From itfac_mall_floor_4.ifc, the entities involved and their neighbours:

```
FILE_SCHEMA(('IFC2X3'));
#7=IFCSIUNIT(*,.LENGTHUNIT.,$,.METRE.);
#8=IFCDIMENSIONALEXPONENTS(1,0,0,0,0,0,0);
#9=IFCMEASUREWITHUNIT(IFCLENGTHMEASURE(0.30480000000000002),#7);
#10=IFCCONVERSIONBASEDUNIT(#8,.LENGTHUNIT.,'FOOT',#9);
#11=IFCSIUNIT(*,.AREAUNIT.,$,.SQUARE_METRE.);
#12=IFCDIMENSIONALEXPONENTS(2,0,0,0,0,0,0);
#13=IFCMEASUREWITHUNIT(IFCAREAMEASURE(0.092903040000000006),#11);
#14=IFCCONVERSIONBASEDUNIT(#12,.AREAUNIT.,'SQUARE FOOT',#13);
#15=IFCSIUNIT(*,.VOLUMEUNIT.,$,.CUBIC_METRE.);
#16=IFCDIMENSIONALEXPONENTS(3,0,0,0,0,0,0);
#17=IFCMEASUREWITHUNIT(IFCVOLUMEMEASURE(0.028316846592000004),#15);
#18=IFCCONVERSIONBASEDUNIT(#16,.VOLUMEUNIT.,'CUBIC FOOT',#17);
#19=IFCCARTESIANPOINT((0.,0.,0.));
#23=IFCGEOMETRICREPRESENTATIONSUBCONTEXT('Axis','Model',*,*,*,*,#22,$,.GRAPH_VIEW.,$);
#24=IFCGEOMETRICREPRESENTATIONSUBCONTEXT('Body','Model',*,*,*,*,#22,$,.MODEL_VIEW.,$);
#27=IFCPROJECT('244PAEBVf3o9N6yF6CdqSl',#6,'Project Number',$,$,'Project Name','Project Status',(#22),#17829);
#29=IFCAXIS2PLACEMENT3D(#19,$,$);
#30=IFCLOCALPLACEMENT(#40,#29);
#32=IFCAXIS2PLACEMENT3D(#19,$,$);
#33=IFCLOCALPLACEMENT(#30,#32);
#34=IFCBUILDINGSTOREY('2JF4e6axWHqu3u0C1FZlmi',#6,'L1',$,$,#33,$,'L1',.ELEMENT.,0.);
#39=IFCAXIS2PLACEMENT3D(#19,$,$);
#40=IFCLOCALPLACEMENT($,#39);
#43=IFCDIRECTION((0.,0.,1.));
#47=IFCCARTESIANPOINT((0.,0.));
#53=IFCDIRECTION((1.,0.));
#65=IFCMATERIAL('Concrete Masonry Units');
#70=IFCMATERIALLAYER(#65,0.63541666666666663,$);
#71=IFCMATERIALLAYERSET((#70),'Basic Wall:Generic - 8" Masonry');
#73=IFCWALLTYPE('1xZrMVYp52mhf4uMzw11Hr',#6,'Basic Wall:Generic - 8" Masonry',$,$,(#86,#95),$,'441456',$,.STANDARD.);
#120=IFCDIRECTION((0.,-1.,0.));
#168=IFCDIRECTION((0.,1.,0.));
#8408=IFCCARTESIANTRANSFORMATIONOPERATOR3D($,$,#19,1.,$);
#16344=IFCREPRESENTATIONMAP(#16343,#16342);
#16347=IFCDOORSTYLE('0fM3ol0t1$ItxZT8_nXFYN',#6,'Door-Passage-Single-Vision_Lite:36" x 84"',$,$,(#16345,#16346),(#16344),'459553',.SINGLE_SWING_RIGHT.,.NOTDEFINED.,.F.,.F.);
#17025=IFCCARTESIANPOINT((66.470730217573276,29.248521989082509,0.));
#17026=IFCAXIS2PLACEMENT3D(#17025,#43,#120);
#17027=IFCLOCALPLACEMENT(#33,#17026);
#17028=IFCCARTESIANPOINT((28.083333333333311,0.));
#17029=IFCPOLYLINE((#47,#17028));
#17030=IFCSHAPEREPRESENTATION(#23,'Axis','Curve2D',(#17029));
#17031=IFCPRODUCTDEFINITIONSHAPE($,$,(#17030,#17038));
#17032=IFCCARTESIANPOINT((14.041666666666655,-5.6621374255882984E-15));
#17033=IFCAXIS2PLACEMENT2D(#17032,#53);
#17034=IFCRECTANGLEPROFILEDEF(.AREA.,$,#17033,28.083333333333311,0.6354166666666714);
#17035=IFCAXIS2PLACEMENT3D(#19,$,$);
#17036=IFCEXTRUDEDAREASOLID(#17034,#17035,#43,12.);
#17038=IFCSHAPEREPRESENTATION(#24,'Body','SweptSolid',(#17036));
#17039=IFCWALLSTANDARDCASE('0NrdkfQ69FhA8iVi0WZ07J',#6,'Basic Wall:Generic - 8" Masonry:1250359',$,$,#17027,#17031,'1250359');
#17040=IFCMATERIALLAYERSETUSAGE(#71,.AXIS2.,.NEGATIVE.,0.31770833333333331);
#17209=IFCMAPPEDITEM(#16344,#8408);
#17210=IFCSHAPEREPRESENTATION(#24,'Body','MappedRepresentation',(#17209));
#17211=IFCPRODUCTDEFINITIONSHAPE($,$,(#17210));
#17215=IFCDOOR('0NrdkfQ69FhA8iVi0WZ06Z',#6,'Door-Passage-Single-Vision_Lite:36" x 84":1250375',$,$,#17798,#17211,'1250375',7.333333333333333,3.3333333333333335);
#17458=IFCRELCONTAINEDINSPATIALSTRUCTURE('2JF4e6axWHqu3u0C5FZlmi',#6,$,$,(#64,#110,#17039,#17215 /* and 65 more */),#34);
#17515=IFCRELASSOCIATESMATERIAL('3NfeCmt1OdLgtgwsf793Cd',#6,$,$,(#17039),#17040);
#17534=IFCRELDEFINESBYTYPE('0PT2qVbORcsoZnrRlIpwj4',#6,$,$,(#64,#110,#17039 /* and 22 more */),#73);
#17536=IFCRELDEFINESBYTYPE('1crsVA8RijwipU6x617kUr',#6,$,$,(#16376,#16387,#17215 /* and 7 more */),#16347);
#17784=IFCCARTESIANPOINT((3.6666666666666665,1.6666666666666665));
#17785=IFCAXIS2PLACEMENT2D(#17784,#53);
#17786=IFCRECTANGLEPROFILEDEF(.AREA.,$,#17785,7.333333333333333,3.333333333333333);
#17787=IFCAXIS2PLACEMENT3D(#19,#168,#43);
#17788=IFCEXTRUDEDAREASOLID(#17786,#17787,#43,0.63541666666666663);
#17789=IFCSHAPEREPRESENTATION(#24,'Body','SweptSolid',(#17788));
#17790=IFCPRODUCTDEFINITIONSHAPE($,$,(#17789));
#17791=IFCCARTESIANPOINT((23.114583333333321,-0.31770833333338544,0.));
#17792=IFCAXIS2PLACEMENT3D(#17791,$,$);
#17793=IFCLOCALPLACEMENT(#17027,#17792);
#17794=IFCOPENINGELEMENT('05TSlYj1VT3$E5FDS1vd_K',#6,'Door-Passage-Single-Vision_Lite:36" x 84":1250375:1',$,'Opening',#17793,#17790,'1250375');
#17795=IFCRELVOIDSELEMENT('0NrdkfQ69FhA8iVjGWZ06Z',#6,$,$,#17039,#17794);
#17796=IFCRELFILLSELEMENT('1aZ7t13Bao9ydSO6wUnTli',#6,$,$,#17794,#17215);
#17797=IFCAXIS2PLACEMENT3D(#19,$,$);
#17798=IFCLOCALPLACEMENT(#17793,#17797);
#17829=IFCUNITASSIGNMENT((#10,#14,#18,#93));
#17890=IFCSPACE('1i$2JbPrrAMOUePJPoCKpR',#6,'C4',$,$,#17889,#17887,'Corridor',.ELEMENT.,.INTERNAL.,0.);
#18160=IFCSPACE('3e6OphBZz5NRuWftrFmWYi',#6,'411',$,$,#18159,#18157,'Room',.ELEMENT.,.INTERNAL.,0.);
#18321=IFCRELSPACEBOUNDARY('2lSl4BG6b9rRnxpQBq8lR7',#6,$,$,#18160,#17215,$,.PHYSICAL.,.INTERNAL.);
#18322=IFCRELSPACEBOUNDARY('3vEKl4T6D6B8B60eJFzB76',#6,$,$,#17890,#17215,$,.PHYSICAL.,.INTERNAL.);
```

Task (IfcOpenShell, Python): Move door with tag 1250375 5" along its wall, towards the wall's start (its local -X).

```python
import ifcopenshell
import ifcopenshell.api.geometry
import ifcopenshell.util.placement
import ifcopenshell.util.unit

model = ifcopenshell.open("itfac_mall_floor_4.ifc")
unit_scale = ifcopenshell.util.unit.calculate_unit_scale(model)

door = model.by_guid("0NrdkfQ69FhA8iVi0WZ06Z")
opening = door.FillsVoids[0].RelatingOpeningElement
wall = opening.VoidsElements[0].RelatingBuildingElement

wall_matrix = ifcopenshell.util.placement.get_local_placement(wall.ObjectPlacement)
shift = wall_matrix[:3, 0] * -5 * 0.0254 / unit_scale
before = ifcopenshell.util.placement.get_local_placement(door.ObjectPlacement)[:3, 3].copy()

# The door is placed relative to its opening, so it follows when the opening moves.
matrix = ifcopenshell.util.placement.get_local_placement(opening.ObjectPlacement)
matrix[:3, 3] += shift
ifcopenshell.api.geometry.edit_object_placement(
    model, product=opening, matrix=matrix, is_si=False, should_transform_children=True
)

after = ifcopenshell.util.placement.get_local_placement(door.ObjectPlacement)[:3, 3]
print("door moved by", (after - before).round(3) + 0.0)

model.write("itfac_mall_floor_4-out.ifc")
```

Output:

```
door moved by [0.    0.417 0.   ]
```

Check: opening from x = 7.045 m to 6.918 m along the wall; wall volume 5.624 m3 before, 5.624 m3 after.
